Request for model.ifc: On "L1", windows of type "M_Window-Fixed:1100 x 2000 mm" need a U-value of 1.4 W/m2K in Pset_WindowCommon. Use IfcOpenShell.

First a look at what the model holds.

```python
import ifcopenshell
import ifcopenshell.util.element

model = ifcopenshell.open("model.ifc")
print(model.schema)
storey = next(s for s in model.by_type("IfcBuildingStorey") if s.Name == "L1")
windows = [e for e in ifcopenshell.util.element.get_decomposition(storey) if e.is_a("IfcWindow")]
seen = {}
for e in windows:
    element_type = ifcopenshell.util.element.get_type(e)
    key = (element_type.Name if element_type != e and element_type else None, ifcopenshell.util.element.get_pset(e, "Pset_WindowCommon", "ThermalTransmittance"))
    seen[key] = seen.get(key, 0) + 1
for (name, value), count in sorted(seen.items(), key=str):
    print(count, "x", name, "|", value)
```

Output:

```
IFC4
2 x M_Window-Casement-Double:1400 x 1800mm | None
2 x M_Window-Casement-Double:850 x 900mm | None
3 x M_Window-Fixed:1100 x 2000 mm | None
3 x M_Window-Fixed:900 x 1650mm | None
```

```python
import ifcopenshell
import ifcopenshell.api.pset
import ifcopenshell.util.element

model = ifcopenshell.open("model.ifc")

storey = next(s for s in model.by_type("IfcBuildingStorey") if s.Name == "L1")
windows = [e for e in ifcopenshell.util.element.get_decomposition(storey) if e.is_a("IfcWindow")]

count = 0
for e in windows:
    element_type = ifcopenshell.util.element.get_type(e)
    if element_type in (None, e) or element_type.Name != "M_Window-Fixed:1100 x 2000 mm":
        continue
    # add_pset returns the element's existing set when there is one.
    pset = ifcopenshell.api.pset.add_pset(model, product=e, name="Pset_WindowCommon")
    ifcopenshell.api.pset.edit_pset(model, pset=pset, properties={"ThermalTransmittance": 1.4})
    count += 1

print(count, "windows updated")

model.write("model_edited.ifc")
```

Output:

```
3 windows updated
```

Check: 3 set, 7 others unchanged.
